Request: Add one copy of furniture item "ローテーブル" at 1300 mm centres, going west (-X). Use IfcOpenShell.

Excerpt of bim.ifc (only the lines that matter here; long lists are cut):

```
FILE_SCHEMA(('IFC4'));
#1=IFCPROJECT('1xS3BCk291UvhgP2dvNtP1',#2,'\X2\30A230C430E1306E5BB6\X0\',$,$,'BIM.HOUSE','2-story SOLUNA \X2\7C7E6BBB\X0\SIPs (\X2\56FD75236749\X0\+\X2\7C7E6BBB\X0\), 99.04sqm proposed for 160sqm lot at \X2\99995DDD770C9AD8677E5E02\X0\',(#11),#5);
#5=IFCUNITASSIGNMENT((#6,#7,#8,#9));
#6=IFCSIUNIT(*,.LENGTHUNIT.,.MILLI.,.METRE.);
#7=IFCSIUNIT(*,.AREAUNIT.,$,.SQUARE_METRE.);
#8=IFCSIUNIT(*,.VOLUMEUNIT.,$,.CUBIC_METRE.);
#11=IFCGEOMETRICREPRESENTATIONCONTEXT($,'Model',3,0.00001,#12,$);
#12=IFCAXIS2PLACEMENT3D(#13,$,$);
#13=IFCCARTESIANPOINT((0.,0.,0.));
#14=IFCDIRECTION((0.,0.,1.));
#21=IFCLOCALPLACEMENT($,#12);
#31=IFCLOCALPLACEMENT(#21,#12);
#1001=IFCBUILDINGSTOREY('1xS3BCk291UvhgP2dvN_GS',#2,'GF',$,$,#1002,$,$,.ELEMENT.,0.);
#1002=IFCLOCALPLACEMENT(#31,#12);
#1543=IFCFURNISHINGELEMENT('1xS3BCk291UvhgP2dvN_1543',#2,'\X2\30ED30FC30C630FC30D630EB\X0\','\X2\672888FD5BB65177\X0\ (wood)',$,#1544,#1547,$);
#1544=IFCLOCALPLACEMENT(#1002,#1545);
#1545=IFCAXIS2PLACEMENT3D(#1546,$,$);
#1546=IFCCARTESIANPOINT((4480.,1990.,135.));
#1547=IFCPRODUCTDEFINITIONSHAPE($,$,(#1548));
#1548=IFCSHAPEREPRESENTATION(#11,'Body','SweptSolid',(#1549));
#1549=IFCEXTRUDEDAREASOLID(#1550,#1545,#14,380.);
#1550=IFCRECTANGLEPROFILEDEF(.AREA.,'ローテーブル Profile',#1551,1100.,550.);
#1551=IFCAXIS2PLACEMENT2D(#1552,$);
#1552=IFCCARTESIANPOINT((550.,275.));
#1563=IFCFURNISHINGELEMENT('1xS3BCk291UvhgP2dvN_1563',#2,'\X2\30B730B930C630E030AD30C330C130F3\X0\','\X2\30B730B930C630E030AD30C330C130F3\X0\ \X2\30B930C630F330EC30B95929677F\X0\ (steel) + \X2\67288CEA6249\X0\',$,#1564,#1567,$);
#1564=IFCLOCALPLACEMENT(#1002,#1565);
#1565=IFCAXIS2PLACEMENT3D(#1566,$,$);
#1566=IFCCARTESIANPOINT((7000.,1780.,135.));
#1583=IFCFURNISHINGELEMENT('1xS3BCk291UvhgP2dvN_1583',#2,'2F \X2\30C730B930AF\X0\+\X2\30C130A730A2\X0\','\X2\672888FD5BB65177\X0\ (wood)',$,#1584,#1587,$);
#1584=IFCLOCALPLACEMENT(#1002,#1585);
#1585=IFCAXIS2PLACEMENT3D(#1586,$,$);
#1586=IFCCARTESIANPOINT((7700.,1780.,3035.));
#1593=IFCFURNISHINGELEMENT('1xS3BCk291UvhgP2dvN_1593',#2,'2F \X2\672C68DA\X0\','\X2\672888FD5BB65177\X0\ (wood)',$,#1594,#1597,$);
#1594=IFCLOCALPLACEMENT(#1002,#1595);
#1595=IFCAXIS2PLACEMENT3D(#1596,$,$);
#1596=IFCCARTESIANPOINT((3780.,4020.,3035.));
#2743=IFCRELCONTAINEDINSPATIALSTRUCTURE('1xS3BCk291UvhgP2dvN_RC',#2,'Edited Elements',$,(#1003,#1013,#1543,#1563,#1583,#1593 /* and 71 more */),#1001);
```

```python
import numpy as np
import ifcopenshell
import ifcopenshell.api.geometry
import ifcopenshell.api.root
import ifcopenshell.util.element
import ifcopenshell.util.placement
import ifcopenshell.util.unit

model = ifcopenshell.open("bim.ifc")
unit_scale = ifcopenshell.util.unit.calculate_unit_scale(model)


def reuse_history(source, copy):
    """copy_class also copies each property set's owner history, people and application; keep the originals."""
    for rel in copy.IsDefinedBy:
        if rel.is_a("IfcRelDefinesByProperties") and (history := rel.RelatingPropertyDefinition.OwnerHistory):
            rel.RelatingPropertyDefinition.OwnerHistory = source.OwnerHistory
            ifcopenshell.util.element.remove_deep2(model, history)


source = model.by_guid("1xS3BCk291UvhgP2dvN_1543")
base = ifcopenshell.util.placement.get_local_placement(source.ObjectPlacement)
step = np.array([-1.0, 0.0, 0.0]) * 1.3 / unit_scale

for i in range(1, 2):
    copy = ifcopenshell.api.root.copy_class(model, product=source)
    copy.Representation = ifcopenshell.util.element.copy_deep(
        model, source.Representation, exclude=["IfcGeometricRepresentationContext", "IfcRepresentationMap"]
    )
    reuse_history(source, copy)
    matrix = base.copy()
    matrix[:3, 3] += i * step
    print("added at", matrix[:3, 3].round(3) + 0.0)
    ifcopenshell.api.geometry.edit_object_placement(model, product=copy, matrix=matrix, is_si=False)

model.write("bim_updated.ifc")
```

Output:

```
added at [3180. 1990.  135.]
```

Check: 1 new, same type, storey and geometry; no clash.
